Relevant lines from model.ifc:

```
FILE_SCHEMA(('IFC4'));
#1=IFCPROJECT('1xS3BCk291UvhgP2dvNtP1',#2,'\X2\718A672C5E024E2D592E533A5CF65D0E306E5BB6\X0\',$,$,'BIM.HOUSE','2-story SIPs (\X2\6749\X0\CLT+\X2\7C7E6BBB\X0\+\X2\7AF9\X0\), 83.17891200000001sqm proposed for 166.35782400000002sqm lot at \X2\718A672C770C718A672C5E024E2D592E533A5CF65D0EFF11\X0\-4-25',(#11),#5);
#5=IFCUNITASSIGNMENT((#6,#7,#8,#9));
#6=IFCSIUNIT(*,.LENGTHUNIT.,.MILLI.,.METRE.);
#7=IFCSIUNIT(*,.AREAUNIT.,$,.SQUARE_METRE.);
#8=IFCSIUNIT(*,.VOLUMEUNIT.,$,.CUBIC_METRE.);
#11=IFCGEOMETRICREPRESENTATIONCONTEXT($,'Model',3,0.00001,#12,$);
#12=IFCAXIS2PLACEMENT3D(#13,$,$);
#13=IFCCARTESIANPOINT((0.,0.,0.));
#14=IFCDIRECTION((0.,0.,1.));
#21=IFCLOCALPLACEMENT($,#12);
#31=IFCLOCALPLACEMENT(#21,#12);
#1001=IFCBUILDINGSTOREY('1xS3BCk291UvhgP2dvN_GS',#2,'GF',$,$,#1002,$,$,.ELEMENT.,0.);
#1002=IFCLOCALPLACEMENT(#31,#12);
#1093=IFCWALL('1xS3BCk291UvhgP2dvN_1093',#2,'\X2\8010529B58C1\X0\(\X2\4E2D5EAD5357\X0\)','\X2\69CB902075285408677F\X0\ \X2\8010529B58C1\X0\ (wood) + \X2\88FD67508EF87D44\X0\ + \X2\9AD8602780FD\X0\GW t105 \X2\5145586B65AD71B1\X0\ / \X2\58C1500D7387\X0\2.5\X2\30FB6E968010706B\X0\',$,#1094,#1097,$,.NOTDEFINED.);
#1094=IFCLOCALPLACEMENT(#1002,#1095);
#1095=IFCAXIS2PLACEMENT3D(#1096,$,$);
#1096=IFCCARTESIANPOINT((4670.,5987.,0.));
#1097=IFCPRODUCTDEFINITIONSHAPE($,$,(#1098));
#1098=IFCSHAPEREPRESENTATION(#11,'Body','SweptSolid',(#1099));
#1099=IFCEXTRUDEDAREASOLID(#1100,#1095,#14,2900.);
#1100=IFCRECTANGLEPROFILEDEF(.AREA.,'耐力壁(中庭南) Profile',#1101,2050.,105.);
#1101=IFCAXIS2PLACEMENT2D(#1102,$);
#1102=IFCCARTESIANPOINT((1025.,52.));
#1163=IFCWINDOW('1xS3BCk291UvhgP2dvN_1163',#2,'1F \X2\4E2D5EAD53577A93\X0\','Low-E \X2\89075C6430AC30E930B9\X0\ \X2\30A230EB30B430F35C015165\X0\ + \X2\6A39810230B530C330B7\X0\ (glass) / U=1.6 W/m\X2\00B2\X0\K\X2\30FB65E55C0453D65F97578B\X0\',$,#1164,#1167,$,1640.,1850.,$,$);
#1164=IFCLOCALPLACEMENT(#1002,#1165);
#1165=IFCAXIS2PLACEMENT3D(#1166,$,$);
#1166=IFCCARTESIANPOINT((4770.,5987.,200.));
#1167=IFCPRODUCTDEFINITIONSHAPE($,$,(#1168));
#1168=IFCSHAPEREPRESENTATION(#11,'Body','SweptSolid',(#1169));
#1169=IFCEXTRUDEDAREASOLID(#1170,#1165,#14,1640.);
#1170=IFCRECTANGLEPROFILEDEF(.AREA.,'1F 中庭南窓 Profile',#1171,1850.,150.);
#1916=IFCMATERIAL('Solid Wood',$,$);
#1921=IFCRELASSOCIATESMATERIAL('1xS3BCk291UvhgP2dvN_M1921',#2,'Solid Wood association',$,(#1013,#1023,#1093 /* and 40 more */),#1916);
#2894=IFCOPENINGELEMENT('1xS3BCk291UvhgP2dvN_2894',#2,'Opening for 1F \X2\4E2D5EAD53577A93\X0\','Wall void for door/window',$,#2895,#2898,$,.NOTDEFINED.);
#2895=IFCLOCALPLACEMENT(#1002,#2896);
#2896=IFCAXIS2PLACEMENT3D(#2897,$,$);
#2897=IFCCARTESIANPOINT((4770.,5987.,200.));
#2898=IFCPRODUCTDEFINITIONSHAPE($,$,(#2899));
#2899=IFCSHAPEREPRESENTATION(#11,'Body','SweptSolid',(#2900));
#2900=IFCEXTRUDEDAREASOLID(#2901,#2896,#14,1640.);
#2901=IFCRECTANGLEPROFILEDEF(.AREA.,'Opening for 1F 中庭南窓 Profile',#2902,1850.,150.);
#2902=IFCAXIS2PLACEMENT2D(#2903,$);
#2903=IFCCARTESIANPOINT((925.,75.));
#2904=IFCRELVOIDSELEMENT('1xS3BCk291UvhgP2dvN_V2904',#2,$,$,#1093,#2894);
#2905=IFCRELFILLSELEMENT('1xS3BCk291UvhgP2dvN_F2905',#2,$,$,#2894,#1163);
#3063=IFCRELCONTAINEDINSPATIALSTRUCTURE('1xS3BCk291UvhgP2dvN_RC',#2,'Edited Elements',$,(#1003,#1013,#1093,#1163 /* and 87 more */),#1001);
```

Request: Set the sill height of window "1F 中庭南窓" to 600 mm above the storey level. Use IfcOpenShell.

```python
import numpy as np
import ifcopenshell
import ifcopenshell.api.geometry
import ifcopenshell.geom
import ifcopenshell.util.element
import ifcopenshell.util.placement
import ifcopenshell.util.shape
import ifcopenshell.util.unit

model = ifcopenshell.open("model.ifc")
unit_scale = ifcopenshell.util.unit.calculate_unit_scale(model)

window = model.by_guid("1xS3BCk291UvhgP2dvN_1163")
opening = window.FillsVoids[0].RelatingOpeningElement
storey = ifcopenshell.util.element.get_container(window, ifc_class="IfcBuildingStorey")
level = ifcopenshell.util.placement.get_local_placement(storey.ObjectPlacement)[2, 3]

# The opening's origin need not be at the sill, so measure its lowest point.
shape = ifcopenshell.geom.create_shape(ifcopenshell.geom.settings(), opening)
bottom = ifcopenshell.util.shape.get_shape_bottom_elevation(shape, shape.geometry) / unit_scale
dz = level + 600.0 - bottom

shift = np.array([0.0, 0.0, dz])
# The window is not placed relative to its opening, so move both.
for product in (opening, window):
    matrix = ifcopenshell.util.placement.get_local_placement(product.ObjectPlacement)
    matrix[:3, 3] += shift
    ifcopenshell.api.geometry.edit_object_placement(model, product=product, matrix=matrix, is_si=False)

print(f"moved by {dz * unit_scale:+.3f} m")

model.write("model-out.ifc")
```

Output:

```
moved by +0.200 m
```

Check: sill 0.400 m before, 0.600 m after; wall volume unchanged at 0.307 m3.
